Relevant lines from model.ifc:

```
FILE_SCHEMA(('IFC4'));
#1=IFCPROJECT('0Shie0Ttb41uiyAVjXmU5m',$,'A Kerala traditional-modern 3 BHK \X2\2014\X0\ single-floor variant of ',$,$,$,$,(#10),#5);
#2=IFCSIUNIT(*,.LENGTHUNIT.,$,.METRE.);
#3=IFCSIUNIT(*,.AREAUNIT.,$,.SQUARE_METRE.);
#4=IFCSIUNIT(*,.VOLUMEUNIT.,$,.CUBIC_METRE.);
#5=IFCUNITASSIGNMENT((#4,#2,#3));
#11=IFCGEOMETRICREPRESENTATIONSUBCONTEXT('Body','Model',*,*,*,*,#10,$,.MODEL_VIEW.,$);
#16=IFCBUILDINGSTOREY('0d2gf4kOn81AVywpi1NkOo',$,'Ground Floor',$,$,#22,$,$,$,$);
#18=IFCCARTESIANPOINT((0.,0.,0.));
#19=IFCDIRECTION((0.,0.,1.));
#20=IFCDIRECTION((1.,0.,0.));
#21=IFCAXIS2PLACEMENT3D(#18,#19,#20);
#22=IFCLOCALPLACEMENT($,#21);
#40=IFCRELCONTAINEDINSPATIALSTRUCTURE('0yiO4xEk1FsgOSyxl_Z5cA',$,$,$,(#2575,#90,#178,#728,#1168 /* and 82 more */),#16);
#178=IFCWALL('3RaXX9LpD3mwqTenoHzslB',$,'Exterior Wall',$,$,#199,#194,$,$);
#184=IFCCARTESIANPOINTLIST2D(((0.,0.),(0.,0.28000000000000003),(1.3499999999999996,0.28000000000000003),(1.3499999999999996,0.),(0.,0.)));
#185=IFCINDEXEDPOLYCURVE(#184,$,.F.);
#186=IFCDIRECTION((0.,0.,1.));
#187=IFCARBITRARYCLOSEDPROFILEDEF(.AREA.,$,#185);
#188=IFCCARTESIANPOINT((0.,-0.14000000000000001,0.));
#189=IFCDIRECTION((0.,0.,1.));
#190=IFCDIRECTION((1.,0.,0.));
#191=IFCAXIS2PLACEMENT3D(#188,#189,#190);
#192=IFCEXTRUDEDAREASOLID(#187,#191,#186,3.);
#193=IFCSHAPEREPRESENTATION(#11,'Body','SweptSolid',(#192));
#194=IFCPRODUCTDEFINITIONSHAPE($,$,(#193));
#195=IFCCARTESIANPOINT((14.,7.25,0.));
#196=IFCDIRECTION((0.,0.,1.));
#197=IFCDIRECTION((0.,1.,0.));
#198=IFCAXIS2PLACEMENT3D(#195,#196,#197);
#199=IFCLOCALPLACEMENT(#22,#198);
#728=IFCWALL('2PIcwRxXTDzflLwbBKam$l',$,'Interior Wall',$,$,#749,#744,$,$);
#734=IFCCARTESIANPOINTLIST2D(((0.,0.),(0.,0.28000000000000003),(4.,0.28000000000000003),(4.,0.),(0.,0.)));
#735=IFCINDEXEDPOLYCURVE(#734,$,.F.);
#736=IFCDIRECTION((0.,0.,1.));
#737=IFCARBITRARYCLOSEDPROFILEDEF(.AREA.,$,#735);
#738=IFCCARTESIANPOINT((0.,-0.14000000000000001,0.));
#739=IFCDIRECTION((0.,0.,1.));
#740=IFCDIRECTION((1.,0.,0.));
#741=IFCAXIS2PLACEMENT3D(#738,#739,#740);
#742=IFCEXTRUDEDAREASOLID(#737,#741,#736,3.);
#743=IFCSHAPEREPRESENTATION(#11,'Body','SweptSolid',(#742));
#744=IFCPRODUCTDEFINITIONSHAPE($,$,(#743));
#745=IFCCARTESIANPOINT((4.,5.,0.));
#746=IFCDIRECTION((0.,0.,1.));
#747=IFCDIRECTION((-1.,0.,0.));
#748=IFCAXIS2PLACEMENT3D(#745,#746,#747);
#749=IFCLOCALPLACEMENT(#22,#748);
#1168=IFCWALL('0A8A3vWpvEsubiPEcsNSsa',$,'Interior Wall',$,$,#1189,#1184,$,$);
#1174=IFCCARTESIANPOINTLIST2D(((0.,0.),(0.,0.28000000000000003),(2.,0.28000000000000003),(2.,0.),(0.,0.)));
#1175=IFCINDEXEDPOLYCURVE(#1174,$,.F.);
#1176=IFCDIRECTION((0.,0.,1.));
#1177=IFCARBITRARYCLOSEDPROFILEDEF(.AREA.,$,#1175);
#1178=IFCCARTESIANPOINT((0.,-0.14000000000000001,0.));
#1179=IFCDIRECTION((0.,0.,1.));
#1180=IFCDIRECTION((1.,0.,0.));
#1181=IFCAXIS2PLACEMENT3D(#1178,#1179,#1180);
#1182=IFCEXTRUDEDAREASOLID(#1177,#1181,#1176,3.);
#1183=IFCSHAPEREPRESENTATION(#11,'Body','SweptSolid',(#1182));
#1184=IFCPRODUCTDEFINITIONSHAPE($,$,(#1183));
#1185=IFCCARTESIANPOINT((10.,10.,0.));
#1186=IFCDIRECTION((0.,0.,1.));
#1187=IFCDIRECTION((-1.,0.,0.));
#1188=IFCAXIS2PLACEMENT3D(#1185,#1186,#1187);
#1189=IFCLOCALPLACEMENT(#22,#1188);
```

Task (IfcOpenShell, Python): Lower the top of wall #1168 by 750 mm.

```python
import ifcopenshell
import ifcopenshell.geom
import ifcopenshell.util.representation
import ifcopenshell.util.shape
import ifcopenshell.util.unit

model = ifcopenshell.open("model.ifc")
unit_scale = ifcopenshell.util.unit.calculate_unit_scale(model)
settings = ifcopenshell.geom.settings()


def volume(element):
    """Net volume in cubic metres, openings subtracted."""
    shape = ifcopenshell.geom.create_shape(settings, element)
    return ifcopenshell.util.shape.get_volume(shape.geometry)


wall = model.by_guid("0A8A3vWpvEsubiPEcsNSsa")
before = volume(wall)

body = ifcopenshell.util.representation.get_representation(wall, "Model", "Body")
solid = body.Items[0]
old_height = solid.Depth
solid.Depth -= 0.75 / unit_scale
after = volume(wall)

print(f"height {old_height:g} -> {solid.Depth:g}, volume {before:.3f} -> {after:.3f} m3")

model.write("model_updated.ifc")
```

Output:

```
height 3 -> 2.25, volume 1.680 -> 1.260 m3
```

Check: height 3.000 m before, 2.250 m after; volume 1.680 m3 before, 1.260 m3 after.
